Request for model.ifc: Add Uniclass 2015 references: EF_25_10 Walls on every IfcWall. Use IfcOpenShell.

First a look at what the model holds.

```python
import ifcopenshell

model = ifcopenshell.open("model.ifc")
print(model.schema)
print("classifications:", [c.Name for c in model.by_type("IfcClassification")])
for ifc_class in ("IfcDoor", "IfcRoof", "IfcStair", "IfcWall", "IfcWindow"):
    print(ifc_class, len(model.by_type(ifc_class)))
```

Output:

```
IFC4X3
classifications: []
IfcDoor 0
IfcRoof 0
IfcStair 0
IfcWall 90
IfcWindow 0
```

```python
import ifcopenshell
import ifcopenshell.api.classification

model = ifcopenshell.open("model.ifc")

system = ifcopenshell.api.classification.add_classification(model, classification="Uniclass 2015")

codes = {
    "IfcWall": ("EF_25_10", "Walls"),
}
for ifc_class, (code, name) in codes.items():
    products = model.by_type(ifc_class)
    ifcopenshell.api.classification.add_reference(
        model, products=products, classification=system, identification=code, name=name
    )
    print(code, len(products))

model.write("model_rev.ifc")
```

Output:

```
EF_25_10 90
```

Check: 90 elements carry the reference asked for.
